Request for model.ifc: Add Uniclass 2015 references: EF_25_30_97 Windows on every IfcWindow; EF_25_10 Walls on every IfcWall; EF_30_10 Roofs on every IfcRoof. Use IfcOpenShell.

First a look at what the model holds.

```python
import ifcopenshell

model = ifcopenshell.open("model.ifc")
print(model.schema)
print("classifications:", [c.Name for c in model.by_type("IfcClassification")])
for ifc_class in ("IfcDoor", "IfcRoof", "IfcStair", "IfcWall", "IfcWindow"):
    print(ifc_class, len(model.by_type(ifc_class)))
```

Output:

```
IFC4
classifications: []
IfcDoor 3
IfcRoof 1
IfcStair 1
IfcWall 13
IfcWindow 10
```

```python
import ifcopenshell
import ifcopenshell.api.classification

model = ifcopenshell.open("model.ifc")

system = ifcopenshell.api.classification.add_classification(model, classification="Uniclass 2015")

codes = {
    "IfcWindow": ("EF_25_30_97", "Windows"),
    "IfcWall": ("EF_25_10", "Walls"),
    "IfcRoof": ("EF_30_10", "Roofs"),
}
for ifc_class, (code, name) in codes.items():
    products = model.by_type(ifc_class)
    ifcopenshell.api.classification.add_reference(
        model, products=products, classification=system, identification=code, name=name
    )
    print(code, len(products))

model.write("model-out.ifc")
```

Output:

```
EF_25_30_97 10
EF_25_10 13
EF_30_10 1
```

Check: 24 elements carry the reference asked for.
